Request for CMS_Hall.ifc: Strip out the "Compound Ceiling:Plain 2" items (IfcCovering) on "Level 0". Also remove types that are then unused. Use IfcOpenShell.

First a look at what the model holds.

```python
import ifcopenshell
import ifcopenshell.util.element

model = ifcopenshell.open("CMS_Hall.ifc")
print(model.schema)
storey = next(s for s in model.by_type("IfcBuildingStorey") if s.Name == "Level 0")
coverings = [e for e in ifcopenshell.util.element.get_decomposition(storey) if e.is_a("IfcCovering")]
seen = {}
for e in coverings:
    element_type = ifcopenshell.util.element.get_type(e)
    name = element_type.Name if element_type not in (None, e) else None
    seen[name] = seen.get(name, 0) + 1
for name, count in sorted(seen.items(), key=str):
    print(count, "x", name)
```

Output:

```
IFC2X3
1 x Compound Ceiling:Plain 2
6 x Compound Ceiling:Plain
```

```python
import ifcopenshell
import ifcopenshell.api.root
import ifcopenshell.util.element

model = ifcopenshell.open("CMS_Hall.ifc")

storey = next(s for s in model.by_type("IfcBuildingStorey") if s.Name == "Level 0")
coverings = [e for e in ifcopenshell.util.element.get_decomposition(storey) if e.is_a("IfcCovering")]
targets = [e for e in coverings if (t := ifcopenshell.util.element.get_type(e)) not in (None, e) and t.Name == "Compound Ceiling:Plain 2"]
types = {ifcopenshell.util.element.get_type(e) for e in targets} - {None, *targets}

for e in targets:
    ifcopenshell.api.root.remove_product(model, product=e)
print(len(targets), "removed")

unused = [t for t in types if not ifcopenshell.util.element.get_types(t)]
for t in unused:
    ifcopenshell.api.root.remove_product(model, product=t)
print(len(unused), "unused types removed")

model.write("CMS_Hall_v2.ifc")
```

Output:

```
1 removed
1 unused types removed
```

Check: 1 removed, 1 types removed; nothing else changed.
